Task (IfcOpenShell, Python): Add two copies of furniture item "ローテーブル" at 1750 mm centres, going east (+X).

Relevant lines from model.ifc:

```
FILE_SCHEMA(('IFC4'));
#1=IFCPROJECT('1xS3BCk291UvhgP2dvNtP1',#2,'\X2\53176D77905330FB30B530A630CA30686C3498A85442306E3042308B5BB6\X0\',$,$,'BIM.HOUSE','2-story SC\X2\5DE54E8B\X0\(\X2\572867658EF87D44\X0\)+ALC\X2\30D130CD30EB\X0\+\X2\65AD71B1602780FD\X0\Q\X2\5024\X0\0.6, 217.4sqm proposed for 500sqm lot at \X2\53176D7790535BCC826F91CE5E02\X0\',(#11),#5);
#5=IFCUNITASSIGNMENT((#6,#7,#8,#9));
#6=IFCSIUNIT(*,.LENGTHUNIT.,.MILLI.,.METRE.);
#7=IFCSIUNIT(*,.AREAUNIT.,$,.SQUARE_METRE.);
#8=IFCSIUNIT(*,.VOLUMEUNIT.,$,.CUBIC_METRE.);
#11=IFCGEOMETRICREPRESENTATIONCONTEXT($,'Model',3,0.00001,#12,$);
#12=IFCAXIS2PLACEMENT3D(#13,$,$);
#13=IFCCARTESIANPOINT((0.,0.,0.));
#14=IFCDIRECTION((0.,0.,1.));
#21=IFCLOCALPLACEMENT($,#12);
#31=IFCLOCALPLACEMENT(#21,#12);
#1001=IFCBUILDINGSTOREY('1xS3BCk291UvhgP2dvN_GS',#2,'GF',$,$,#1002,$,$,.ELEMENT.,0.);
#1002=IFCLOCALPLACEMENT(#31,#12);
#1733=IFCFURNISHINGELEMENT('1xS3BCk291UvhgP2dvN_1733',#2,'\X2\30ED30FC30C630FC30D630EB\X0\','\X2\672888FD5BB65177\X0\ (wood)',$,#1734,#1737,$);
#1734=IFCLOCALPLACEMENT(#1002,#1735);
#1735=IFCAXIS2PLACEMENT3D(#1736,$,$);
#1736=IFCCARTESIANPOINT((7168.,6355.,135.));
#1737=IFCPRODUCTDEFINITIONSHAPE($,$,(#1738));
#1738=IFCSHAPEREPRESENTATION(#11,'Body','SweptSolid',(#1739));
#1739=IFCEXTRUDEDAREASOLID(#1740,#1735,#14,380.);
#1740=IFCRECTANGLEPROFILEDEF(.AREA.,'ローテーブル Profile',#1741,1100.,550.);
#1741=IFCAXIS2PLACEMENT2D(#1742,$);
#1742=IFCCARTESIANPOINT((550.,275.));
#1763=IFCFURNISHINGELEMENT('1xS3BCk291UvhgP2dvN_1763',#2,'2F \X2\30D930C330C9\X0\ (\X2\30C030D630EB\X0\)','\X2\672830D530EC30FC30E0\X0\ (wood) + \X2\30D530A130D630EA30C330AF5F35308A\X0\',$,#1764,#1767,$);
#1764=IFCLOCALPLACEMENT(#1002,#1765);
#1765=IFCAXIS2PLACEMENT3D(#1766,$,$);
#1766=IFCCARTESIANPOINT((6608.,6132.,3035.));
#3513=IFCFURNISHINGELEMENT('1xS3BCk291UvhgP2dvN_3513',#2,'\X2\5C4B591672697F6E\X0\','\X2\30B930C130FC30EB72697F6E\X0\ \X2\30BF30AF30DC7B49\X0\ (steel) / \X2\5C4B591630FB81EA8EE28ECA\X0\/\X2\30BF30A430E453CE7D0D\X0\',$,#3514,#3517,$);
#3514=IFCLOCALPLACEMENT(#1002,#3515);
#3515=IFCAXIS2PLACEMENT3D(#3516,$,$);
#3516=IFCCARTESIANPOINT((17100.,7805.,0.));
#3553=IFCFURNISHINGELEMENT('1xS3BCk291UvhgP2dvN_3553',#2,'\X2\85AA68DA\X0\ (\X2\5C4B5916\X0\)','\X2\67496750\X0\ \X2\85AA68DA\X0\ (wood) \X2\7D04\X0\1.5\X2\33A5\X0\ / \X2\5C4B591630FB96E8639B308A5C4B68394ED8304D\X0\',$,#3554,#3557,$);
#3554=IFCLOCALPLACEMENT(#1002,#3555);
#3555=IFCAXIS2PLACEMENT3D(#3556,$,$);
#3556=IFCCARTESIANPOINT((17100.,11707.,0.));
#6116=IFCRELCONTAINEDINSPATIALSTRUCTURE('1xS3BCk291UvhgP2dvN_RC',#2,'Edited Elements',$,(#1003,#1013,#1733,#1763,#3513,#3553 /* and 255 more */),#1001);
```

```python
import numpy as np
import ifcopenshell
import ifcopenshell.api.geometry
import ifcopenshell.api.root
import ifcopenshell.util.element
import ifcopenshell.util.placement

model = ifcopenshell.open("model.ifc")


def reuse_history(source, copy):
    """copy_class also copies each property set's owner history, people and application; keep the originals."""
    for rel in copy.IsDefinedBy:
        if rel.is_a("IfcRelDefinesByProperties") and (history := rel.RelatingPropertyDefinition.OwnerHistory):
            rel.RelatingPropertyDefinition.OwnerHistory = source.OwnerHistory
            ifcopenshell.util.element.remove_deep2(model, history)


source = model.by_id(1733)
base = ifcopenshell.util.placement.get_local_placement(source.ObjectPlacement)
step = np.array([1.0, 0.0, 0.0]) * 1750.0

for i in range(1, 3):
    copy = ifcopenshell.api.root.copy_class(model, product=source)
    copy.Representation = ifcopenshell.util.element.copy_deep(
        model, source.Representation, exclude=["IfcGeometricRepresentationContext", "IfcRepresentationMap"]
    )
    reuse_history(source, copy)
    matrix = base.copy()
    matrix[:3, 3] += i * step
    print("added at", matrix[:3, 3].round(3) + 0.0)
    ifcopenshell.api.geometry.edit_object_placement(model, product=copy, matrix=matrix, is_si=False)

model.write("model_v2.ifc")
```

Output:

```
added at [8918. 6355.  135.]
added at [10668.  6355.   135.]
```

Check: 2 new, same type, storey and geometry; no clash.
